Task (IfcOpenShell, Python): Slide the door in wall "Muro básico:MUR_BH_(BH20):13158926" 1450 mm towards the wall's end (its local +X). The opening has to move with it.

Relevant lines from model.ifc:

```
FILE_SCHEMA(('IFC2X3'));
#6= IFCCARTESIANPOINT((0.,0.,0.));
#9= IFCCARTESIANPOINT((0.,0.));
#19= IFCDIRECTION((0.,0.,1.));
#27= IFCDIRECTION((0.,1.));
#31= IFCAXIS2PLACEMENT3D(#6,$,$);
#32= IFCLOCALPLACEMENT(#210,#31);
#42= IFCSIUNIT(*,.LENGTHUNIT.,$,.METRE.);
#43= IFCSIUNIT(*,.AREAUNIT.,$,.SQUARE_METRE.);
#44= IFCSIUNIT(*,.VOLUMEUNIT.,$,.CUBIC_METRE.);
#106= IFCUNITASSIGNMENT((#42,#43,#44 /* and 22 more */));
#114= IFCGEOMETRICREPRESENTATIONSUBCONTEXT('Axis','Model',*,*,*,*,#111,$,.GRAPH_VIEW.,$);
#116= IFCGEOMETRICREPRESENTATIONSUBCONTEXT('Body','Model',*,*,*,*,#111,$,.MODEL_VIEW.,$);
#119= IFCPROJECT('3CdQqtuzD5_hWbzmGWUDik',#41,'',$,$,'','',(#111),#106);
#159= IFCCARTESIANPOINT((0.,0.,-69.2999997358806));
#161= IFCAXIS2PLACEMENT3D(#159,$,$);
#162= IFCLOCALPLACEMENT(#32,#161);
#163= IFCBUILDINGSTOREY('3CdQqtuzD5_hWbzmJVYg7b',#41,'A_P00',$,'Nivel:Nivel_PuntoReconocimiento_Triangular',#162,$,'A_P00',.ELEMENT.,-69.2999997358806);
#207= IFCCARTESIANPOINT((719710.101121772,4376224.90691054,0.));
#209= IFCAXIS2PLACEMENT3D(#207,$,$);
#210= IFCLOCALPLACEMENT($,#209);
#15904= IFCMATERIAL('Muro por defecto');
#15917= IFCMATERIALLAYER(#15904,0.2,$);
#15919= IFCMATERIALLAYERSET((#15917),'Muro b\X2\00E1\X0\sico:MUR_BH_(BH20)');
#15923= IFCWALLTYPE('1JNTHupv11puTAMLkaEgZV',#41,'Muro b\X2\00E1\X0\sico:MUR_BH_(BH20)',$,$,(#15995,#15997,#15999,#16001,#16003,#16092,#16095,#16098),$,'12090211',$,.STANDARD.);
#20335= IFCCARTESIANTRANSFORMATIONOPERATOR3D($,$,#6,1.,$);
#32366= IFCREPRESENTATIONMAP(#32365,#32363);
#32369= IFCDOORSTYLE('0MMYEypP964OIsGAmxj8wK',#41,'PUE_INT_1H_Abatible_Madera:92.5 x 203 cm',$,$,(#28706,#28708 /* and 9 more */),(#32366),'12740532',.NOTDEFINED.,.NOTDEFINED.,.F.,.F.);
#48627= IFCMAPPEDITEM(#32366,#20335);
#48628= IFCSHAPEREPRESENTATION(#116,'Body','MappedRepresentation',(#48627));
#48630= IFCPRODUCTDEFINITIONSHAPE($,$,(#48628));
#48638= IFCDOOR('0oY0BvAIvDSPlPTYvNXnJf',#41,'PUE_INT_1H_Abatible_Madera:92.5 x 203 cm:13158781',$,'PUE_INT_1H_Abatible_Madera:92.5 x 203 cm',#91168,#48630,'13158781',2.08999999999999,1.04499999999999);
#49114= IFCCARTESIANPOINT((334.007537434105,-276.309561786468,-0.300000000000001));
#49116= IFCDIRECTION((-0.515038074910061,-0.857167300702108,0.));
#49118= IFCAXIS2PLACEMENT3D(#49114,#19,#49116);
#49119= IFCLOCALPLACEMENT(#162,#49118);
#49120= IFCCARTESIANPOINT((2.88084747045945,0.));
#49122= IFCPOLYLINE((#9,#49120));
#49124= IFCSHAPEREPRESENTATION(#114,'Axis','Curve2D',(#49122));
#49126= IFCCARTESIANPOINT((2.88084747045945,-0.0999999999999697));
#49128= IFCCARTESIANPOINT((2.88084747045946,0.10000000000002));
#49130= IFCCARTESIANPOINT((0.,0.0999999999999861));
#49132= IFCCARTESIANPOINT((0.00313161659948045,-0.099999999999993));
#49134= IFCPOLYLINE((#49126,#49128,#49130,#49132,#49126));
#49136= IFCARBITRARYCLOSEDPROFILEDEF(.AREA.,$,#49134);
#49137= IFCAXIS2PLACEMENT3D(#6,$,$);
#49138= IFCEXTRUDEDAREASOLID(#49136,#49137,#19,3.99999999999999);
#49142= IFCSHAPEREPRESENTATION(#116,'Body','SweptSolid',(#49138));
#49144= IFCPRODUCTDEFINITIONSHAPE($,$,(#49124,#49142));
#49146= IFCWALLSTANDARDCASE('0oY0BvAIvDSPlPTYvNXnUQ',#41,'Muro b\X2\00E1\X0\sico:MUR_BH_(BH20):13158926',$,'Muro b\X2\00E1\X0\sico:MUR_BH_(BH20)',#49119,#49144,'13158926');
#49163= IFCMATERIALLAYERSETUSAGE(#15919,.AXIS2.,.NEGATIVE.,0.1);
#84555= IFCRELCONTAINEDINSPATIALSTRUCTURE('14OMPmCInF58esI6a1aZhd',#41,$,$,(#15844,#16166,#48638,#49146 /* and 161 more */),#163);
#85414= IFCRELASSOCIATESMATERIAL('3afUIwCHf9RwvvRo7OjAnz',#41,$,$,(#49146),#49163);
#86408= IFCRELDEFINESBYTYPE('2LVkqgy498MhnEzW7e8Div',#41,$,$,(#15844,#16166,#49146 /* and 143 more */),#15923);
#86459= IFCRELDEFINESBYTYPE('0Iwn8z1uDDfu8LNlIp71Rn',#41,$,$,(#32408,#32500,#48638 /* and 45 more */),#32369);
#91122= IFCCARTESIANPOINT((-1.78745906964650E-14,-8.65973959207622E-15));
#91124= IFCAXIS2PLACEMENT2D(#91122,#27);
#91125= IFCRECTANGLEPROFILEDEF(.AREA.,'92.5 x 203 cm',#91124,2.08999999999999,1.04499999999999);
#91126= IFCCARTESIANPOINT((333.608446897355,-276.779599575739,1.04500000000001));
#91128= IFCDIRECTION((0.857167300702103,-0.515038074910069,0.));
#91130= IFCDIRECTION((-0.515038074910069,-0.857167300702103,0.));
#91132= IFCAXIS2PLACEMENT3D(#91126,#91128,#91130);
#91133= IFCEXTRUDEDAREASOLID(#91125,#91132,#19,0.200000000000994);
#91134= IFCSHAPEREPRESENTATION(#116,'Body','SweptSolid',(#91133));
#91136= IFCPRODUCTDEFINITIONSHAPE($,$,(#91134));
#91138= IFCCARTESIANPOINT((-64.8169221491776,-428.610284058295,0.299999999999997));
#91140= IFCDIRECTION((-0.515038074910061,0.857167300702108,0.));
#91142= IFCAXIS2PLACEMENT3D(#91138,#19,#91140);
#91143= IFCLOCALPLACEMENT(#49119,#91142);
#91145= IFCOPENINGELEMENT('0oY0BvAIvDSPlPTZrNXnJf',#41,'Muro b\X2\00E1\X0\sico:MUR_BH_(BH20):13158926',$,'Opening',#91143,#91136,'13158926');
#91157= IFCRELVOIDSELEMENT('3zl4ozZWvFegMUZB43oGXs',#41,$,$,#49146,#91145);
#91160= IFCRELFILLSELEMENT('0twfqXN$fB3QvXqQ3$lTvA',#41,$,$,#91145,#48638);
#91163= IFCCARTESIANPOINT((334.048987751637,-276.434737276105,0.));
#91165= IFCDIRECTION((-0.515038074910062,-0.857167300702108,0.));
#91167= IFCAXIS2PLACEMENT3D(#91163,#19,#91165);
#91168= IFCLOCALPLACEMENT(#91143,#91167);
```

```python
import ifcopenshell
import ifcopenshell.api.geometry
import ifcopenshell.util.placement

model = ifcopenshell.open("model.ifc")

door = model.by_id(48638)
opening = door.FillsVoids[0].RelatingOpeningElement
wall = opening.VoidsElements[0].RelatingBuildingElement

wall_matrix = ifcopenshell.util.placement.get_local_placement(wall.ObjectPlacement)
shift = wall_matrix[:3, 0] * 1.45
before = ifcopenshell.util.placement.get_local_placement(door.ObjectPlacement)[:3, 3].copy()

# The door is placed relative to its opening, so it follows when the opening moves.
matrix = ifcopenshell.util.placement.get_local_placement(opening.ObjectPlacement)
matrix[:3, 3] += shift
ifcopenshell.api.geometry.edit_object_placement(
    model, product=opening, matrix=matrix, is_si=False, should_transform_children=True
)

after = ifcopenshell.util.placement.get_local_placement(door.ObjectPlacement)[:3, 3]
print("door moved by", (after - before).round(3) + 0.0)

model.write("model_v2.ifc")
```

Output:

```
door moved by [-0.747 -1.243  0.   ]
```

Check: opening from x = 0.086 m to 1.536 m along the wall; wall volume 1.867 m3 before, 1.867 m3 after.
